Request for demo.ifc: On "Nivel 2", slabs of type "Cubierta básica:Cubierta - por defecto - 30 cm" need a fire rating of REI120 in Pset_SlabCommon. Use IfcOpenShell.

First a look at what the model holds.

```python
import ifcopenshell
import ifcopenshell.util.element

model = ifcopenshell.open("demo.ifc")
print(model.schema)
storey = next(s for s in model.by_type("IfcBuildingStorey") if s.Name == "Nivel 2")
slabs = [e for e in ifcopenshell.util.element.get_decomposition(storey) if e.is_a("IfcSlab")]
seen = {}
for e in slabs:
    element_type = ifcopenshell.util.element.get_type(e)
    key = (element_type.Name if element_type != e and element_type else None, ifcopenshell.util.element.get_pset(e, "Pset_SlabCommon", "FireRating"))
    seen[key] = seen.get(key, 0) + 1
for (name, value), count in sorted(seen.items(), key=str):
    print(count, "x", name, "|", value)
```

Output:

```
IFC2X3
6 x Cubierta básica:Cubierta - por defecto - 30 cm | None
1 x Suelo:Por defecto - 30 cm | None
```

```python
import ifcopenshell
import ifcopenshell.api.pset
import ifcopenshell.util.element

model = ifcopenshell.open("demo.ifc")

storey = next(s for s in model.by_type("IfcBuildingStorey") if s.Name == "Nivel 2")
slabs = [e for e in ifcopenshell.util.element.get_decomposition(storey) if e.is_a("IfcSlab")]

count = 0
for e in slabs:
    element_type = ifcopenshell.util.element.get_type(e)
    if element_type in (None, e) or element_type.Name != "Cubierta básica:Cubierta - por defecto - 30 cm":
        continue
    # add_pset returns the element's existing set when there is one.
    pset = ifcopenshell.api.pset.add_pset(model, product=e, name="Pset_SlabCommon")
    ifcopenshell.api.pset.edit_pset(model, pset=pset, properties={"FireRating": "REI120"})
    count += 1

print(count, "slabs updated")

model.write("demo_rev.ifc")
```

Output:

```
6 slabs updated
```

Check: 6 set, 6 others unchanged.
